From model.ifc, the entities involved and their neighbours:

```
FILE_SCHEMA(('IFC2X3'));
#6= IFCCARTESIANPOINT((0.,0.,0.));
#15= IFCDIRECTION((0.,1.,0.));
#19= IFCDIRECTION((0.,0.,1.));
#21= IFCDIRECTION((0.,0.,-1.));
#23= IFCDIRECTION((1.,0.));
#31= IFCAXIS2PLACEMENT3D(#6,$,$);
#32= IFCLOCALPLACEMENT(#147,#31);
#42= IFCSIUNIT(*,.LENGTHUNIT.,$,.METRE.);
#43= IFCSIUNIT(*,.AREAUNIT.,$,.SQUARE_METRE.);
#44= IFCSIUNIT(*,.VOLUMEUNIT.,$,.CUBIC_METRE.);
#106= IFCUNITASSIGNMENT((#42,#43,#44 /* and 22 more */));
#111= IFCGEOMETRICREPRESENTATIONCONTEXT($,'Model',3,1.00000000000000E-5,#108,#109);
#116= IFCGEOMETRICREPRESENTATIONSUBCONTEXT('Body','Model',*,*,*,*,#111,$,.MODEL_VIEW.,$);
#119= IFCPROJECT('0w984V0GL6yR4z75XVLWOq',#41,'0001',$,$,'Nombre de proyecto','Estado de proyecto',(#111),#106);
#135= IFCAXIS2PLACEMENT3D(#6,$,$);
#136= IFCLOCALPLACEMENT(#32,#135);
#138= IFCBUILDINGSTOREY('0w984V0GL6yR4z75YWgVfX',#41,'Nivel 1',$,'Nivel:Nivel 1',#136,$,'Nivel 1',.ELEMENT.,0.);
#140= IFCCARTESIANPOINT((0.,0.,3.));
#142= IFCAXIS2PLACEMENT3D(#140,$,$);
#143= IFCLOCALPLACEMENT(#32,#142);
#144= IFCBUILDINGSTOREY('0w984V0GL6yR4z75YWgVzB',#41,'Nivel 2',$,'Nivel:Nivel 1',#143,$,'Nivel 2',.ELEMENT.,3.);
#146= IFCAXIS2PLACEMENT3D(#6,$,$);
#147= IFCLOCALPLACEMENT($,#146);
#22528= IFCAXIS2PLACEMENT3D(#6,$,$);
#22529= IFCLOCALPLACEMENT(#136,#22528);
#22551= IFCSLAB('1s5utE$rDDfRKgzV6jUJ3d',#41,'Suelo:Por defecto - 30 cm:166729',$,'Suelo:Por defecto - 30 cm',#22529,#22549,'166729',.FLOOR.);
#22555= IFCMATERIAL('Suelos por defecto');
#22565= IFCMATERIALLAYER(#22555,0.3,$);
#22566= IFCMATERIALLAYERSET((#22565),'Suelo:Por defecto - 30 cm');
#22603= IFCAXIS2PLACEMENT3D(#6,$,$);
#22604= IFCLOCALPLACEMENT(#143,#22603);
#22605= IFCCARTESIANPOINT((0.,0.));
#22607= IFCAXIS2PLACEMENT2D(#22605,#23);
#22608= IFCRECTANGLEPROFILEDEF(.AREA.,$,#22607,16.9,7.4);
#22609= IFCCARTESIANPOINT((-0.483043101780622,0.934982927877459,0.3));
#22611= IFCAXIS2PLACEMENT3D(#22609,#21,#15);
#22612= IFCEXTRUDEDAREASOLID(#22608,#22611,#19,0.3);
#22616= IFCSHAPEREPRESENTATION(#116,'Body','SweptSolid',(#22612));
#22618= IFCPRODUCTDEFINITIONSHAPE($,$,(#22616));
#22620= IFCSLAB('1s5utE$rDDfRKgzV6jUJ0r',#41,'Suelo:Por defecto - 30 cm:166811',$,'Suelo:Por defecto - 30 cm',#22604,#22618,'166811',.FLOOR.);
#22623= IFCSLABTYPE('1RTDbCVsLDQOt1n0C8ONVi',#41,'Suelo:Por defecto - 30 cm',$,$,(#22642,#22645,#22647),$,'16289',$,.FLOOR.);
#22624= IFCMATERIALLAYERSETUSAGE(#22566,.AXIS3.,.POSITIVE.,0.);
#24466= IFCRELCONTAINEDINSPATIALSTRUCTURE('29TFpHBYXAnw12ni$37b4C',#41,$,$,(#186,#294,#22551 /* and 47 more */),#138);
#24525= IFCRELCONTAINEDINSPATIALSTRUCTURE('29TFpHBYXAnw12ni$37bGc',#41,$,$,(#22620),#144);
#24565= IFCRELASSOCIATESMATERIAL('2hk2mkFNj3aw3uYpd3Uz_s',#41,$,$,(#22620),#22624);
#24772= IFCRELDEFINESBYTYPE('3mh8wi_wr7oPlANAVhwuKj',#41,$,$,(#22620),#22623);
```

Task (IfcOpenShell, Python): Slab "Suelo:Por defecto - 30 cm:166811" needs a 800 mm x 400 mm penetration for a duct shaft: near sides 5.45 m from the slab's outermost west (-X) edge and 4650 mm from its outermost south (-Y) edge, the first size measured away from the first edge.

```python
import numpy as np
import ifcopenshell
import ifcopenshell.api.feature
import ifcopenshell.api.geometry
import ifcopenshell.api.root
import ifcopenshell.geom
import ifcopenshell.util.placement
import ifcopenshell.util.representation
import ifcopenshell.util.shape
import ifcopenshell.util.unit

model = ifcopenshell.open("model.ifc")
unit_scale = ifcopenshell.util.unit.calculate_unit_scale(model)
settings = ifcopenshell.geom.settings()


def volume(element):
    """Net volume in cubic metres, openings subtracted."""
    shape = ifcopenshell.geom.create_shape(settings, element)
    return ifcopenshell.util.shape.get_volume(shape.geometry)


slab = model.by_guid("1s5utE$rDDfRKgzV6jUJ0r")
before = volume(slab)

# Extent in the slab's own axes, in metres. The edges named are its -X and -Y sides.
slab_shape = ifcopenshell.geom.create_shape(settings, slab)
vertices = ifcopenshell.util.shape.get_vertices(slab_shape.geometry)
x_min, y_min, bottom = vertices.min(axis=0)
top = vertices[:, 2].max()

opening = ifcopenshell.api.root.create_entity(model, ifc_class="IfcOpeningElement", name="Duct shaft opening")
context = ifcopenshell.util.representation.get_context(model, "Model", "Body", "MODEL_VIEW")
width, depth = 0.8, 0.4
outline = [(0.0, 0.0), (width, 0.0), (width, depth), (0.0, depth), (0.0, 0.0)]
# Overshoot both faces by 50 mm so the cut is clean.
shape = ifcopenshell.api.geometry.add_slab_representation(
    model, context=context, depth=top - bottom + 0.1, polyline=outline
)
ifcopenshell.api.geometry.assign_representation(model, product=opening, representation=shape)

matrix = ifcopenshell.util.placement.get_local_placement(slab.ObjectPlacement)
matrix[:, 3] = matrix @ np.append(np.array([x_min + 5.45, y_min + 4.65, bottom - 0.05]) / unit_scale, 1.0)
ifcopenshell.api.geometry.edit_object_placement(model, product=opening, matrix=matrix, is_si=False)
ifcopenshell.api.feature.add_feature(model, feature=opening, element=slab)

after = volume(slab)

print(f"slab volume {before:.3f} -> {after:.3f} m3")

model.write("model-out.ifc")
```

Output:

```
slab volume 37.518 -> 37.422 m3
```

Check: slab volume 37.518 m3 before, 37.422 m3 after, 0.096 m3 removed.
